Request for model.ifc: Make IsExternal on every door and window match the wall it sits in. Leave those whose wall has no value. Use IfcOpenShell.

First a look at what the model holds.

```python
import ifcopenshell
import ifcopenshell.util.element

model = ifcopenshell.open("model.ifc")
print(model.schema)
seen = {}
for e in model.by_type("IfcDoor") + model.by_type("IfcWindow"):
    if not e.FillsVoids:
        continue
    host = e.FillsVoids[0].RelatingOpeningElement.VoidsElements[0].RelatingBuildingElement
    own = ifcopenshell.util.element.get_pset(e, f"Pset_{e.is_a()[3:].removesuffix('StandardCase')}Common", "IsExternal")
    wall = ifcopenshell.util.element.get_pset(host, "Pset_WallCommon", "IsExternal")
    seen[e.is_a(), own, wall] = seen.get((e.is_a(), own, wall), 0) + 1
for (cls, own, wall), count in sorted(seen.items(), key=str):
    print(count, cls, "IsExternal:", own, "| host wall:", wall)
```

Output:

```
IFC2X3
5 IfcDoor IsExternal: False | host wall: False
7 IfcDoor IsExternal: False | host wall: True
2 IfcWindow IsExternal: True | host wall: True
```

```python
import ifcopenshell
import ifcopenshell.api.pset
import ifcopenshell.util.element

model = ifcopenshell.open("model.ifc")

count = 0
for ifc_class, pset_name in (("IfcDoor", "Pset_DoorCommon"), ("IfcWindow", "Pset_WindowCommon")):
    for e in model.by_type(ifc_class):
        if not e.FillsVoids:
            continue
        host = e.FillsVoids[0].RelatingOpeningElement.VoidsElements[0].RelatingBuildingElement
        external = ifcopenshell.util.element.get_pset(host, "Pset_WallCommon", "IsExternal")
        if external is None or ifcopenshell.util.element.get_pset(e, pset_name, "IsExternal") == external:
            continue
        pset = ifcopenshell.api.pset.add_pset(model, product=e, name=pset_name)
        ifcopenshell.api.pset.edit_pset(model, pset=pset, properties={"IsExternal": external})
        count += 1

print(count, "updated")

model.write("model_updated.ifc")
```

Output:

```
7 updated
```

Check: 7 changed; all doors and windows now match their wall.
